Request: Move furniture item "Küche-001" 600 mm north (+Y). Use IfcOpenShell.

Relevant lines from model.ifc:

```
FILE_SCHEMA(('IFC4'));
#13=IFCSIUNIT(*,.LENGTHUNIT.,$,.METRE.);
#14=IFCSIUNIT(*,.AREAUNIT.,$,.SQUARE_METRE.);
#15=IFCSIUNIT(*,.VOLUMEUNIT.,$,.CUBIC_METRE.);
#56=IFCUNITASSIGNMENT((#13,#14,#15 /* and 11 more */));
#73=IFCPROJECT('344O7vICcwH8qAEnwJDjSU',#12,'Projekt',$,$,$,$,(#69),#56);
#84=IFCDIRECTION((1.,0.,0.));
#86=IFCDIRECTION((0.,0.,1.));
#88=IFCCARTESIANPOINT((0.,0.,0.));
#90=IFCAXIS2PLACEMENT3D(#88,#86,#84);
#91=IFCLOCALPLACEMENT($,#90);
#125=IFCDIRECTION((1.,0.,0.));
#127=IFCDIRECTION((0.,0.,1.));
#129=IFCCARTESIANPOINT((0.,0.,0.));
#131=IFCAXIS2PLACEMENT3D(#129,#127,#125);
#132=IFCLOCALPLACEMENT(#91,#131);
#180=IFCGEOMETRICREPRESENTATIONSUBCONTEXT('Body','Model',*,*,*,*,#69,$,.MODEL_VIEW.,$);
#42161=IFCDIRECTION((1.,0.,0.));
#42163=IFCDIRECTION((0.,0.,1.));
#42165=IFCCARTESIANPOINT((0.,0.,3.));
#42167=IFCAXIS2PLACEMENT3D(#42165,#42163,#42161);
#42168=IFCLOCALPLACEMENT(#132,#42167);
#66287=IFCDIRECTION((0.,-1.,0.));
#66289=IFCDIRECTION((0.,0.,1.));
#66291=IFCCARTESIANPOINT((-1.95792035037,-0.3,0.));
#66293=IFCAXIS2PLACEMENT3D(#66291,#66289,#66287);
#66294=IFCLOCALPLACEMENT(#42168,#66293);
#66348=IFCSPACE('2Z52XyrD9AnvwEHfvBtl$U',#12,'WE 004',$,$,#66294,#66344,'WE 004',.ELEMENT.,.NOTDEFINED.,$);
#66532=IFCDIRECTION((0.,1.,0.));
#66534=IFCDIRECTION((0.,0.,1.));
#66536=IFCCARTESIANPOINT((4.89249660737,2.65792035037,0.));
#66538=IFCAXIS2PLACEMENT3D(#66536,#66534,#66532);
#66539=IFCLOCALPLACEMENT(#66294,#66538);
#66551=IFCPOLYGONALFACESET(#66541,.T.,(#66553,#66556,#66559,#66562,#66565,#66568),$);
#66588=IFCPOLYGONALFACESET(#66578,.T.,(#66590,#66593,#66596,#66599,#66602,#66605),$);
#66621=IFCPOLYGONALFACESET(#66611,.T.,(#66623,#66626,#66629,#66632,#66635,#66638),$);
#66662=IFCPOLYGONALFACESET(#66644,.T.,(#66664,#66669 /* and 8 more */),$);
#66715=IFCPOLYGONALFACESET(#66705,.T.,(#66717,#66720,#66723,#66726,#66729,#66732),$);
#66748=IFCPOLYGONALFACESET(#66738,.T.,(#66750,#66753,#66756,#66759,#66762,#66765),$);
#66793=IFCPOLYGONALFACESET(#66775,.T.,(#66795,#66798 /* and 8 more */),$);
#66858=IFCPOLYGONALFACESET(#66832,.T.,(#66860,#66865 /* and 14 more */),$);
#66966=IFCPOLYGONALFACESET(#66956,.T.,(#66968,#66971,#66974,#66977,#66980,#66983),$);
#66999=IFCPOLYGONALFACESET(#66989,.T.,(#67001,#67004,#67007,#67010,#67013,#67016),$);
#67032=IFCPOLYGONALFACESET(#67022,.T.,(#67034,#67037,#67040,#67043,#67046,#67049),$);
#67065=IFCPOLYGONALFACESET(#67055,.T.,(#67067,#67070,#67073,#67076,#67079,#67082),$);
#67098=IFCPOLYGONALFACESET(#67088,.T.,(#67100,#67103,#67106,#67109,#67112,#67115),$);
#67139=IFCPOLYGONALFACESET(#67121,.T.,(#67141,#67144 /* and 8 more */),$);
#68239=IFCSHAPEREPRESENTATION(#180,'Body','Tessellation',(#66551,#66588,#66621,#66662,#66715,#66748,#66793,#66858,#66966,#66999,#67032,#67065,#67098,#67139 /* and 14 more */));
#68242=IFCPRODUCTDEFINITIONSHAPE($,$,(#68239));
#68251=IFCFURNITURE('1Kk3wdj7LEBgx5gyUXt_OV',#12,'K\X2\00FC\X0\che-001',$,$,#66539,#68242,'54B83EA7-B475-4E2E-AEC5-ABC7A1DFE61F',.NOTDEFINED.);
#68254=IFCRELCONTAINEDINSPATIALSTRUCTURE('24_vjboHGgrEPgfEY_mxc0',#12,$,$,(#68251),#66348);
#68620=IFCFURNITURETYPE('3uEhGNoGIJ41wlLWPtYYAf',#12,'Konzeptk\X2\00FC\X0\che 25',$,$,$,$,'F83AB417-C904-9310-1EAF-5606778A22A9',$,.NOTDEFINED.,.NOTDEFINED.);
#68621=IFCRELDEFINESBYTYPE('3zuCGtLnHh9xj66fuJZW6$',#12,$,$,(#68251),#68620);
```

```python
import ifcopenshell
import ifcopenshell.api.geometry
import ifcopenshell.util.placement

model = ifcopenshell.open("model.ifc")

item = model.by_guid("1Kk3wdj7LEBgx5gyUXt_OV")
matrix = ifcopenshell.util.placement.get_local_placement(item.ObjectPlacement)
matrix[1, 3] += 0.6
ifcopenshell.api.geometry.edit_object_placement(model, product=item, matrix=matrix, is_si=False)

print(ifcopenshell.util.placement.get_local_placement(item.ObjectPlacement).round(3) + 0.0)

model.write("model-out.ifc")
```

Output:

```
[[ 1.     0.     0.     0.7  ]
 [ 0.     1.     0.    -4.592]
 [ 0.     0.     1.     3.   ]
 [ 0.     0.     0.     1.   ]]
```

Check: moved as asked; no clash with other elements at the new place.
